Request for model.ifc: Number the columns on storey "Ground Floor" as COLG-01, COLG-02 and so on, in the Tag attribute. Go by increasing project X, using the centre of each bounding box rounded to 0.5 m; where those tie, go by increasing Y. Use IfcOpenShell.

First a look at what the model holds.

```python
import ifcopenshell
import ifcopenshell.util.element
import ifcopenshell.util.placement

model = ifcopenshell.open("model.ifc")
print(model.schema)
storey = next(s for s in model.by_type("IfcBuildingStorey") if s.Name == "Ground Floor")
columns = [e for e in ifcopenshell.util.element.get_decomposition(storey) if e.is_a("IfcColumn")]
for e in sorted(columns, key=lambda e: e.id()):
    origin = ifcopenshell.util.placement.get_local_placement(e.ObjectPlacement)[:3, 3]
    print(e.id(), e.Tag, e.Name, origin.round(2) + 0.0, sep=" | ")
```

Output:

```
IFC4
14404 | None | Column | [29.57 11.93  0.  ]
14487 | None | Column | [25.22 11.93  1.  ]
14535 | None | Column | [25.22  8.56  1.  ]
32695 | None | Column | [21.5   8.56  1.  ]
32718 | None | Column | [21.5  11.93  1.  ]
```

```python
import ifcopenshell
import ifcopenshell.geom
import ifcopenshell.util.element
import ifcopenshell.util.shape

model = ifcopenshell.open("model.ifc")
settings = ifcopenshell.geom.settings()
settings.set("use-world-coords", True)


def centre(element):
    shape = ifcopenshell.geom.create_shape(settings, element)
    return ifcopenshell.util.shape.get_bbox_centroid(shape.geometry)


storey = next(s for s in model.by_type("IfcBuildingStorey") if s.Name == "Ground Floor")
columns = [e for e in ifcopenshell.util.element.get_decomposition(storey) if e.is_a("IfcColumn")]

# Insertion points can sit at a corner or the storey origin, so sort by the geometry (in metres).
centres = {e: centre(e) for e in columns}
columns.sort(key=lambda e: (round(centres[e][0] / 0.5), centres[e][1]))

for i, e in enumerate(columns, start=1):
    number = f"COLG-{i:02d}"
    e.Tag = number
    print(e.id(), number)

model.write("model_edited.ifc")
```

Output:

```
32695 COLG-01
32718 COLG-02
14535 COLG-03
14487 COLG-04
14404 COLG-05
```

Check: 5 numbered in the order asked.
